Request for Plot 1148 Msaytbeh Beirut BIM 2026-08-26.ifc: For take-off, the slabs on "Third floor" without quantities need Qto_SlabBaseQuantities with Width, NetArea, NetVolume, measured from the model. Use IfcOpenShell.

First a look at what the model holds.

```python
import ifcopenshell
import ifcopenshell.util.element
import ifcopenshell.util.unit

model = ifcopenshell.open("Plot 1148 Msaytbeh Beirut BIM 2026-08-26.ifc")
print(model.schema)
for unit_type in ("LENGTHUNIT", "AREAUNIT", "VOLUMEUNIT"):
    print(unit_type, ifcopenshell.util.unit.calculate_unit_scale(model, unit_type))
storey = next(s for s in model.by_type("IfcBuildingStorey") if s.Name == "Third floor")
slabs = [e for e in ifcopenshell.util.element.get_decomposition(storey) if e.is_a("IfcSlab")]
for e in sorted(slabs, key=lambda e: e.id()):
    print(e.id(), e.is_a(), e.Name, list(ifcopenshell.util.element.get_psets(e, qtos_only=True)), sep=" | ")
```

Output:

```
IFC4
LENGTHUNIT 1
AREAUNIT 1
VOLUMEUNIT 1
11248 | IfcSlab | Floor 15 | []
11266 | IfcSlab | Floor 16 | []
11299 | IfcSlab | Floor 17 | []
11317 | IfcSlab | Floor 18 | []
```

```python
import ifcopenshell
import ifcopenshell.api.pset
import ifcopenshell.geom
import ifcopenshell.util.element
import ifcopenshell.util.shape
import ifcopenshell.util.unit

model = ifcopenshell.open("Plot 1148 Msaytbeh Beirut BIM 2026-08-26.ifc")
unit_scale = ifcopenshell.util.unit.calculate_unit_scale(model)
area_scale = ifcopenshell.util.unit.calculate_unit_scale(model, "AREAUNIT")
volume_scale = ifcopenshell.util.unit.calculate_unit_scale(model, "VOLUMEUNIT")
settings = ifcopenshell.geom.settings()

storey = next(s for s in model.by_type("IfcBuildingStorey") if s.Name == "Third floor")
slabs = [e for e in ifcopenshell.util.element.get_decomposition(storey) if e.is_a("IfcSlab")]

for e in sorted(slabs, key=lambda e: e.id()):
    if ifcopenshell.util.element.get_psets(e, qtos_only=True, should_inherit=False):
        continue
    # Geometry comes back in metres, in the element's own axes.
    shape = ifcopenshell.geom.create_shape(settings, e)
    values = {
        "Width": ifcopenshell.util.shape.get_z(shape.geometry) / unit_scale,
        "NetArea": ifcopenshell.util.shape.get_footprint_area(shape.geometry) / area_scale,
        "NetVolume": ifcopenshell.util.shape.get_volume(shape.geometry) / volume_scale,
    }
    qto = ifcopenshell.api.pset.add_qto(model, product=e, name="Qto_SlabBaseQuantities")
    ifcopenshell.api.pset.edit_qto(model, qto=qto, properties=values)
    print(e.id(), {k: round(v, 3) for k, v in values.items()})

model.write("Plot 1148 Msaytbeh Beirut BIM 2026-08-26_rev.ifc")
```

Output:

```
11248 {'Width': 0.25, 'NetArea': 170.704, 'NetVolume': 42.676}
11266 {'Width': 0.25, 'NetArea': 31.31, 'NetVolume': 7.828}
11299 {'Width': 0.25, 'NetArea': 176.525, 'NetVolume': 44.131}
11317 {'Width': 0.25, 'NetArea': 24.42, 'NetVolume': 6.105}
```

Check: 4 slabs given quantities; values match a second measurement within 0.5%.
